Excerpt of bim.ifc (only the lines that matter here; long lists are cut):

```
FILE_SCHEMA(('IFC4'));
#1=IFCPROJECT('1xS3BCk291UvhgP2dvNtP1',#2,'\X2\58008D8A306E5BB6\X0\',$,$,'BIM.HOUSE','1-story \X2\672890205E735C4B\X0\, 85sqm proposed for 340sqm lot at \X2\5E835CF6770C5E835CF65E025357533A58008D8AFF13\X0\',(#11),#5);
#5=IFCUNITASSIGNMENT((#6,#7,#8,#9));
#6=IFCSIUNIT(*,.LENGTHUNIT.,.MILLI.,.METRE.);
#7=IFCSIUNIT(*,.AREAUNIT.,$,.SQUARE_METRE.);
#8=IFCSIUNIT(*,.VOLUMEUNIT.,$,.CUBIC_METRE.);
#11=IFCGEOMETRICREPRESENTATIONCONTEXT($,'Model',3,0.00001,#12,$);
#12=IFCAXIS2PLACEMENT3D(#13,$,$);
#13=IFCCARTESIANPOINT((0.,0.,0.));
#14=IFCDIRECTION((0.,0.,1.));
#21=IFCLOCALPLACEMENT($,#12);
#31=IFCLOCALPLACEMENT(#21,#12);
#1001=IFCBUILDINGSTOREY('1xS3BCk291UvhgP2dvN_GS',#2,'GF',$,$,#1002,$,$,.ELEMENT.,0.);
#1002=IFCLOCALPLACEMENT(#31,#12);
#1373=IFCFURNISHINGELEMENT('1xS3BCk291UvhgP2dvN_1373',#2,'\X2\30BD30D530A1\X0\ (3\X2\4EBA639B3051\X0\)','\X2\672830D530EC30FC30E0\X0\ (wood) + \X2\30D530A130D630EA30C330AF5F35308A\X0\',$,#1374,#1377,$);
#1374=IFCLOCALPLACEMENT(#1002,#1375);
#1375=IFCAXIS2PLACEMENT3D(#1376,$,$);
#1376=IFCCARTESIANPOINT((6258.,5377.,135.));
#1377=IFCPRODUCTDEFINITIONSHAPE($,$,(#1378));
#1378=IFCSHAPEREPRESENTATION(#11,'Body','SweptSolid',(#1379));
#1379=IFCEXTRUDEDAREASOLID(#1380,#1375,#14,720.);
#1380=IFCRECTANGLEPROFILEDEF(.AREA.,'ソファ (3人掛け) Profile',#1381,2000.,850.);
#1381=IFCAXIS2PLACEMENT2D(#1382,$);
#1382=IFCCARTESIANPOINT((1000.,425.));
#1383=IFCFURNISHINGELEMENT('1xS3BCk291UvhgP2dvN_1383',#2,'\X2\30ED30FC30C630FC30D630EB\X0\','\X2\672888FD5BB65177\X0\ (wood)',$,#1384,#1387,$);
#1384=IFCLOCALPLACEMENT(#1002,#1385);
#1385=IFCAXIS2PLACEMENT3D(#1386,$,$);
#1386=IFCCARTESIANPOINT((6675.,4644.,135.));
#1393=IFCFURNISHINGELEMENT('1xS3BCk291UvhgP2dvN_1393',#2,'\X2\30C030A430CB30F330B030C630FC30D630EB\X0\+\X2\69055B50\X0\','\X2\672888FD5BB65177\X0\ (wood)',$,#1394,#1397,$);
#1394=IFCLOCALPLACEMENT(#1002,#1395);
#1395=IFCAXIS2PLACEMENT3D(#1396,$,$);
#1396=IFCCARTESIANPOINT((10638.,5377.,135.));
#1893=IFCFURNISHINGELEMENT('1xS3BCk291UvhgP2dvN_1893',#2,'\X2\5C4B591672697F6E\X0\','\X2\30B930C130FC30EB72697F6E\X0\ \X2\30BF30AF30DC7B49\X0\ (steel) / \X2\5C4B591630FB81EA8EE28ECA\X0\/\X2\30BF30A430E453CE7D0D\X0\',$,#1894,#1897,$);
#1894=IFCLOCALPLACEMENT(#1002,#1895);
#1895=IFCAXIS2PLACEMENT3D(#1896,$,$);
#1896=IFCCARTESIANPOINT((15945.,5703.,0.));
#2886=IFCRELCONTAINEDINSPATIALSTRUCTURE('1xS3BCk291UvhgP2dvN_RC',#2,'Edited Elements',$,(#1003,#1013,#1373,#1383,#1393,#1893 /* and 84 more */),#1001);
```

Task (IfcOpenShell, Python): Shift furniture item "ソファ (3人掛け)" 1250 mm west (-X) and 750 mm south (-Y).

```python
import ifcopenshell
import ifcopenshell.api.geometry
import ifcopenshell.util.placement

model = ifcopenshell.open("bim.ifc")

item = model.by_id(1373)
matrix = ifcopenshell.util.placement.get_local_placement(item.ObjectPlacement)
matrix[0, 3] -= 1250.0
matrix[1, 3] -= 750.0
ifcopenshell.api.geometry.edit_object_placement(model, product=item, matrix=matrix, is_si=False)

print(ifcopenshell.util.placement.get_local_placement(item.ObjectPlacement).round(3) + 0.0)

model.write("bim_rev.ifc")
```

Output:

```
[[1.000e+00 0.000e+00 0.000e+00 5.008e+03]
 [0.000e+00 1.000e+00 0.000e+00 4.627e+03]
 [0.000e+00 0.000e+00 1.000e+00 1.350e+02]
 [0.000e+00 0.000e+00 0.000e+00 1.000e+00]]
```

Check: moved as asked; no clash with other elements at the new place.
